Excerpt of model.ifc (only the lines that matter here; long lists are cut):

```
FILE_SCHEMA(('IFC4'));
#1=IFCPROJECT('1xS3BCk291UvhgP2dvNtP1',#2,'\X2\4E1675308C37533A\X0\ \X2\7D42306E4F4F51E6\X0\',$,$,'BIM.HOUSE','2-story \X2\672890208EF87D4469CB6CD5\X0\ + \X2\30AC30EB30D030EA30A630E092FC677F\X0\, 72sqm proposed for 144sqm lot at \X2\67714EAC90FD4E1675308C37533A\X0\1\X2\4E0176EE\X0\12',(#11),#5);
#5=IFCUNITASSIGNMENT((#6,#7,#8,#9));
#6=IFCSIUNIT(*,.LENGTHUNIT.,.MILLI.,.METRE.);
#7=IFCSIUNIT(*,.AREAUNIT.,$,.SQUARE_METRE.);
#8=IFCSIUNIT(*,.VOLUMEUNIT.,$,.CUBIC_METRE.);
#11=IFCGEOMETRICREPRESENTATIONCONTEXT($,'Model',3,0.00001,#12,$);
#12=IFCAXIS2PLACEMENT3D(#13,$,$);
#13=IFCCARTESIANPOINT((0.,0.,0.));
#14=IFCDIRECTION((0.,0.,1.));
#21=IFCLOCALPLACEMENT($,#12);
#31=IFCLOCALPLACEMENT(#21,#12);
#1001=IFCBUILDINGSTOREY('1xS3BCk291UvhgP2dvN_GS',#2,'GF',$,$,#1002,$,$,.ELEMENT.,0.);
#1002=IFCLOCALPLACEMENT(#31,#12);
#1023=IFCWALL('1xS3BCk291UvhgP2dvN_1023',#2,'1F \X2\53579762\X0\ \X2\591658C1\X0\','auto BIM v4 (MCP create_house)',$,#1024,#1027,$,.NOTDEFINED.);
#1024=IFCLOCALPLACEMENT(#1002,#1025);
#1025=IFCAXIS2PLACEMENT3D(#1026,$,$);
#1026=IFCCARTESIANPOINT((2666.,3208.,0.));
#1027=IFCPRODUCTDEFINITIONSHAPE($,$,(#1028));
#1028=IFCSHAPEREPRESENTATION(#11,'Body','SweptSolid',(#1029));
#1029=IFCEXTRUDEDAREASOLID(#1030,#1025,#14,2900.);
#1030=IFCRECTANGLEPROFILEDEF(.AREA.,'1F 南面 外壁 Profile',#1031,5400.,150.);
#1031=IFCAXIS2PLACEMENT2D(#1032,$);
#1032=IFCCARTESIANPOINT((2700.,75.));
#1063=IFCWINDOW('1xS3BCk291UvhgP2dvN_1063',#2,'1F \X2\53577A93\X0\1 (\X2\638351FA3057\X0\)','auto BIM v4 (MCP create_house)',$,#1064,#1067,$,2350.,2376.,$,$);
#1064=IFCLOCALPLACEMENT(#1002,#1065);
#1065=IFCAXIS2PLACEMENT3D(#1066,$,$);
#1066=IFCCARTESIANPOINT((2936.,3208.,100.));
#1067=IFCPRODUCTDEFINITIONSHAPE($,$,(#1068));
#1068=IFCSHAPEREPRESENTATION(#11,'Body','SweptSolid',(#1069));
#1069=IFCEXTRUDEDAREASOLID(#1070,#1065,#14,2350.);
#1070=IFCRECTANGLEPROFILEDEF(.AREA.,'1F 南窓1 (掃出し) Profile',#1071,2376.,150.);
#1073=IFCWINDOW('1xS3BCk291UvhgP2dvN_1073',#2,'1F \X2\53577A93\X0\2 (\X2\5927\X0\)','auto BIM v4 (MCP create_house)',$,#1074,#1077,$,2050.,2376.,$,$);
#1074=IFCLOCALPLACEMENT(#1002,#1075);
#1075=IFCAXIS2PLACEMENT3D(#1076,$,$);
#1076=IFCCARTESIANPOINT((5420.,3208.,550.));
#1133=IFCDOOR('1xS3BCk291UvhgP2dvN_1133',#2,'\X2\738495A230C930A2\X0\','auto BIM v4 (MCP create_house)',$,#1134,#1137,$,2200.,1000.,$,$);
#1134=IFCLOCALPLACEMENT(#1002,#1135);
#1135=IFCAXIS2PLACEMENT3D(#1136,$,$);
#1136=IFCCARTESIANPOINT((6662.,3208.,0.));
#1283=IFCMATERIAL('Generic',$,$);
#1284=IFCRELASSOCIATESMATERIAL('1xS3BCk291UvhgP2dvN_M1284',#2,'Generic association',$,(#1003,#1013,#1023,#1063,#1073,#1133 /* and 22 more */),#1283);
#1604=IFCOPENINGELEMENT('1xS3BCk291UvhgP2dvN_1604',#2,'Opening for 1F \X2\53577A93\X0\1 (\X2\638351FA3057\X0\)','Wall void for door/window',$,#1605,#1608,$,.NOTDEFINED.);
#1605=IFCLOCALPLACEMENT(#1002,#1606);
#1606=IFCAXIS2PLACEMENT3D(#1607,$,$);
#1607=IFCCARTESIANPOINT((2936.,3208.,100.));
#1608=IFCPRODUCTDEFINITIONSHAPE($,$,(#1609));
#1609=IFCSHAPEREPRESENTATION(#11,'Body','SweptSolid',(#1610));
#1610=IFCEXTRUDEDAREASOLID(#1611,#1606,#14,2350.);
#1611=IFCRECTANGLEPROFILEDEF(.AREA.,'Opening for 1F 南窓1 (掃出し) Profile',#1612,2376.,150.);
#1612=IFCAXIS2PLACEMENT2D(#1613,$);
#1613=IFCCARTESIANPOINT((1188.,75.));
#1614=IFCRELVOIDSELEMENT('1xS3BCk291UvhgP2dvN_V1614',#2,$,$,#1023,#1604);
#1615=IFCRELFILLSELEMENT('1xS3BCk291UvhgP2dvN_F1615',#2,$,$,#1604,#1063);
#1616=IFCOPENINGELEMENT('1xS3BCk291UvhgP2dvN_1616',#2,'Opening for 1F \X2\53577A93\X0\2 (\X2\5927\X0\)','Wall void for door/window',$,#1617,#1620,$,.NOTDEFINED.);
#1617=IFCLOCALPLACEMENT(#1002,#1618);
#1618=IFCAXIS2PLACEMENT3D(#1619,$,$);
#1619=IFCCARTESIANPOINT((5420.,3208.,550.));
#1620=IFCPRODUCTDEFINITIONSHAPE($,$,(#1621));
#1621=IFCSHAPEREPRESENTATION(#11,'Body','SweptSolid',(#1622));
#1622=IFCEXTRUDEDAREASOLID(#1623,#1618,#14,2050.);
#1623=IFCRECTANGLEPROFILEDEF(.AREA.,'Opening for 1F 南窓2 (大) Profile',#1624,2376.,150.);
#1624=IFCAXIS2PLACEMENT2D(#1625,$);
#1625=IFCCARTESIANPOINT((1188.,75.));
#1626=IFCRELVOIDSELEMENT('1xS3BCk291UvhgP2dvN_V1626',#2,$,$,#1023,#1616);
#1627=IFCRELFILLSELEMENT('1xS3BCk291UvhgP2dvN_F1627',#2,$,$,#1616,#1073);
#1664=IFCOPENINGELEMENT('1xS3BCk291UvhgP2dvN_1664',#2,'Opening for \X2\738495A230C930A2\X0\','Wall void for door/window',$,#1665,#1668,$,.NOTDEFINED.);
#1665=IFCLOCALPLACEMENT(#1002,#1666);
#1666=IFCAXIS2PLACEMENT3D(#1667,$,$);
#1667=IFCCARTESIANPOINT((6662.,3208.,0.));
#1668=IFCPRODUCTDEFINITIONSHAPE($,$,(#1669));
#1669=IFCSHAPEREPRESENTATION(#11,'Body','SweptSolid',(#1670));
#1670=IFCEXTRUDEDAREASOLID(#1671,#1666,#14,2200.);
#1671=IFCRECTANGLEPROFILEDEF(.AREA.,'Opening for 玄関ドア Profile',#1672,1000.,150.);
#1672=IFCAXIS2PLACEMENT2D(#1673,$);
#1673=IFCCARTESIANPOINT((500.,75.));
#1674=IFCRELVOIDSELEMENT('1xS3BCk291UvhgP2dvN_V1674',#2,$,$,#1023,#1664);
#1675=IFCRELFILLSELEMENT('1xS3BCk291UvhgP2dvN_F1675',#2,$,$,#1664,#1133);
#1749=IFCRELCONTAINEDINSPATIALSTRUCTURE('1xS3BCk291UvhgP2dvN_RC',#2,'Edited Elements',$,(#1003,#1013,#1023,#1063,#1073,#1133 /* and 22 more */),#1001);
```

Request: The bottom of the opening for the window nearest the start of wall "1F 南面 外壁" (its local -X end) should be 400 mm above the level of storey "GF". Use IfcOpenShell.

```python
import numpy as np
import ifcopenshell
import ifcopenshell.api.geometry
import ifcopenshell.geom
import ifcopenshell.util.element
import ifcopenshell.util.placement
import ifcopenshell.util.shape
import ifcopenshell.util.unit

model = ifcopenshell.open("model.ifc")
unit_scale = ifcopenshell.util.unit.calculate_unit_scale(model)

window = model.by_id(1063)
opening = window.FillsVoids[0].RelatingOpeningElement
storey = ifcopenshell.util.element.get_container(window, ifc_class="IfcBuildingStorey")
level = ifcopenshell.util.placement.get_local_placement(storey.ObjectPlacement)[2, 3]

# The opening's origin need not be at the sill, so measure its lowest point.
shape = ifcopenshell.geom.create_shape(ifcopenshell.geom.settings(), opening)
bottom = ifcopenshell.util.shape.get_shape_bottom_elevation(shape, shape.geometry) / unit_scale
dz = level + 0.4 / unit_scale - bottom

shift = np.array([0.0, 0.0, dz])
# The window is not placed relative to its opening, so move both.
for product in (opening, window):
    matrix = ifcopenshell.util.placement.get_local_placement(product.ObjectPlacement)
    matrix[:3, 3] += shift
    ifcopenshell.api.geometry.edit_object_placement(model, product=product, matrix=matrix, is_si=False)

print(f"moved by {dz * unit_scale:+.3f} m")

model.write("model_v2.ifc")
```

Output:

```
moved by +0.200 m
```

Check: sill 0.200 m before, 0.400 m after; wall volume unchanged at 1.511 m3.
